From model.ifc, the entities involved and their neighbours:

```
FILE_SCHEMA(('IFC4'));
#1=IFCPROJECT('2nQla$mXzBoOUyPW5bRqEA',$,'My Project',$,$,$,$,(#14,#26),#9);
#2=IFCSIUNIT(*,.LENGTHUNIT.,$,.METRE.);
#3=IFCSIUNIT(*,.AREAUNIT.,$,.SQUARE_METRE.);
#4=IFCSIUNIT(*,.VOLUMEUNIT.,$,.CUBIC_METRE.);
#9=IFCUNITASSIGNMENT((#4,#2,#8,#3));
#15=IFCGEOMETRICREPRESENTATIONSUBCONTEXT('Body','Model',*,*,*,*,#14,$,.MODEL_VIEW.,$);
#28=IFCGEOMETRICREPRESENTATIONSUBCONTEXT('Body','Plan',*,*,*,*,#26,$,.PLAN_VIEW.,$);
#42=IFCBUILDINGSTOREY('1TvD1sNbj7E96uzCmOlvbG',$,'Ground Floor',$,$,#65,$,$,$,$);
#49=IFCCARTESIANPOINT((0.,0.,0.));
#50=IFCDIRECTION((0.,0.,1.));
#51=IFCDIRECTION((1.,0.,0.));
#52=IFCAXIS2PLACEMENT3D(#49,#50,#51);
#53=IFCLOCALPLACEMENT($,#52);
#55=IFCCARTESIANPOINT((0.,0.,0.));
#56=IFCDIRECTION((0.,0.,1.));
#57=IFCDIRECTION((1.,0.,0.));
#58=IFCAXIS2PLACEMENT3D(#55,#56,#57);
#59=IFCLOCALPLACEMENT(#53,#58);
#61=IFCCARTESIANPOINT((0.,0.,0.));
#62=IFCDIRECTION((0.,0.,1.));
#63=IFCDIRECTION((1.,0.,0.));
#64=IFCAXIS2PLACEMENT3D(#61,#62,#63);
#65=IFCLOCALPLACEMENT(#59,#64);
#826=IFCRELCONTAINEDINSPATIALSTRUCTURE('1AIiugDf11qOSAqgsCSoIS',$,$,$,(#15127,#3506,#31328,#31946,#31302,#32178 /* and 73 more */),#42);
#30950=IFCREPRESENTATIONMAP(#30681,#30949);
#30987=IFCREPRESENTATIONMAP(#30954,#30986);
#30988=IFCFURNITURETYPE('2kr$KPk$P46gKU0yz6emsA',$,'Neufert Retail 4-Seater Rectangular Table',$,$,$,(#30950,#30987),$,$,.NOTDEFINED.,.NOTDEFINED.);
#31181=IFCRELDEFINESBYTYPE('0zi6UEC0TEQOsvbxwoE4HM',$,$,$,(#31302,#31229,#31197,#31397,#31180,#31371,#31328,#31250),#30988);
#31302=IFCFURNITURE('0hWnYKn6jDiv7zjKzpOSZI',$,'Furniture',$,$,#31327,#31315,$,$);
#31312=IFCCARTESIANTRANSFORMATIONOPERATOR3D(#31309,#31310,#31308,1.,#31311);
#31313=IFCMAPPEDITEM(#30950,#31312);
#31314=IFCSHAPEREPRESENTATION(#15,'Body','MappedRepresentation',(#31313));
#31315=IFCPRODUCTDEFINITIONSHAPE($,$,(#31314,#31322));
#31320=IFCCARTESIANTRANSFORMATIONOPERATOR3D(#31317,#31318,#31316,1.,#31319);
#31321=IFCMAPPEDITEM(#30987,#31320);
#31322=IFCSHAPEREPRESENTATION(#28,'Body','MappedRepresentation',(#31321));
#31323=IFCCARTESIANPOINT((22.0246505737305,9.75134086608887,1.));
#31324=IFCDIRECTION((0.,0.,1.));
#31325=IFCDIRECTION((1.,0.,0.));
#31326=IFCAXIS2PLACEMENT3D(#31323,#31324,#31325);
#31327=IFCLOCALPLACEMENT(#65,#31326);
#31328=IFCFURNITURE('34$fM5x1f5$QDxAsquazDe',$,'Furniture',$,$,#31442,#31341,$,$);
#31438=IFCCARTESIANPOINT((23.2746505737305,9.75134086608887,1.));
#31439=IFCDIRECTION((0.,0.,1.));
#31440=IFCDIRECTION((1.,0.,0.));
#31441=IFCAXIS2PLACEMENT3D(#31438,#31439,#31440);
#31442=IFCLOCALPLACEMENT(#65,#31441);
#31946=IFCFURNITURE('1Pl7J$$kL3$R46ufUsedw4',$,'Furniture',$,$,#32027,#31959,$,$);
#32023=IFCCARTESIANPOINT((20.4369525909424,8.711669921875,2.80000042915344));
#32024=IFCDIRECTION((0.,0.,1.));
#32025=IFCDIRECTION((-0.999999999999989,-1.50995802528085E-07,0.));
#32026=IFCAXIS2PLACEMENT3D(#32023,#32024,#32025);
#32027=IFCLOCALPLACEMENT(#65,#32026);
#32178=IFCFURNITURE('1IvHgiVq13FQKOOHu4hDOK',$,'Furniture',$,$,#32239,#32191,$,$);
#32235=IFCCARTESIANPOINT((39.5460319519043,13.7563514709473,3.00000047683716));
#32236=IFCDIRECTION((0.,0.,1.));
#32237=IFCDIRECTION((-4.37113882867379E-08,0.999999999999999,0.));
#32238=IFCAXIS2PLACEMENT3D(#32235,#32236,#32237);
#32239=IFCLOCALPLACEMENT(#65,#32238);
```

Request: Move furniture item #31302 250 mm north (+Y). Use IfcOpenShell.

```python
import ifcopenshell
import ifcopenshell.api.geometry
import ifcopenshell.util.placement
import ifcopenshell.util.unit

model = ifcopenshell.open("model.ifc")
unit_scale = ifcopenshell.util.unit.calculate_unit_scale(model)

item = model.by_guid("0hWnYKn6jDiv7zjKzpOSZI")
matrix = ifcopenshell.util.placement.get_local_placement(item.ObjectPlacement)
matrix[1, 3] += 0.25 / unit_scale
ifcopenshell.api.geometry.edit_object_placement(model, product=item, matrix=matrix, is_si=False)

print(ifcopenshell.util.placement.get_local_placement(item.ObjectPlacement).round(3) + 0.0)

model.write("model_rev.ifc")
```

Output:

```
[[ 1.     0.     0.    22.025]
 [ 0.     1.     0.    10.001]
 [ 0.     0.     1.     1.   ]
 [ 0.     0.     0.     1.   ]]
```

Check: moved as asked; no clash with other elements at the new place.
